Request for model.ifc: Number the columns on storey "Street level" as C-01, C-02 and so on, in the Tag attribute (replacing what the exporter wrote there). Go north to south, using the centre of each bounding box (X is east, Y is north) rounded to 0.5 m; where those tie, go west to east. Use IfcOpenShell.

First a look at what the model holds.

```python
import ifcopenshell
import ifcopenshell.util.element
import ifcopenshell.util.placement

model = ifcopenshell.open("model.ifc")
print(model.schema)
storey = next(s for s in model.by_type("IfcBuildingStorey") if s.Name == "Street level")
columns = [e for e in ifcopenshell.util.element.get_decomposition(storey) if e.is_a("IfcColumn")]
for e in sorted(columns, key=lambda e: e.id()):
    origin = ifcopenshell.util.placement.get_local_placement(e.ObjectPlacement)[:3, 3]
    print(e.id(), e.Tag, e.Name, origin.round(2) + 0.0, sep=" | ")
```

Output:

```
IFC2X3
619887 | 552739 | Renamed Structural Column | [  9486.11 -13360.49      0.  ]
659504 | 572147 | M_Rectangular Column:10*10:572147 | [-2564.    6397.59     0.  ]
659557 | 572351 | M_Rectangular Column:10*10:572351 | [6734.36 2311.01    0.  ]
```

```python
import ifcopenshell
import ifcopenshell.geom
import ifcopenshell.util.element
import ifcopenshell.util.shape

model = ifcopenshell.open("model.ifc")
settings = ifcopenshell.geom.settings()
settings.set("use-world-coords", True)


def centre(element):
    shape = ifcopenshell.geom.create_shape(settings, element)
    return ifcopenshell.util.shape.get_bbox_centroid(shape.geometry)


storey = next(s for s in model.by_type("IfcBuildingStorey") if s.Name == "Street level")
columns = [e for e in ifcopenshell.util.element.get_decomposition(storey) if e.is_a("IfcColumn")]

# Insertion points can sit at a corner or the storey origin, so sort by the geometry (in metres).
centres = {e: centre(e) for e in columns}
columns.sort(key=lambda e: (-round(centres[e][1] / 0.5), centres[e][0]))

for i, e in enumerate(columns, start=1):
    number = f"C-{i:02d}"
    e.Tag = number
    print(e.id(), number)

model.write("model_v2.ifc")
```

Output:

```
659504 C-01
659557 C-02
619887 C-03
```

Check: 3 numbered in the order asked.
